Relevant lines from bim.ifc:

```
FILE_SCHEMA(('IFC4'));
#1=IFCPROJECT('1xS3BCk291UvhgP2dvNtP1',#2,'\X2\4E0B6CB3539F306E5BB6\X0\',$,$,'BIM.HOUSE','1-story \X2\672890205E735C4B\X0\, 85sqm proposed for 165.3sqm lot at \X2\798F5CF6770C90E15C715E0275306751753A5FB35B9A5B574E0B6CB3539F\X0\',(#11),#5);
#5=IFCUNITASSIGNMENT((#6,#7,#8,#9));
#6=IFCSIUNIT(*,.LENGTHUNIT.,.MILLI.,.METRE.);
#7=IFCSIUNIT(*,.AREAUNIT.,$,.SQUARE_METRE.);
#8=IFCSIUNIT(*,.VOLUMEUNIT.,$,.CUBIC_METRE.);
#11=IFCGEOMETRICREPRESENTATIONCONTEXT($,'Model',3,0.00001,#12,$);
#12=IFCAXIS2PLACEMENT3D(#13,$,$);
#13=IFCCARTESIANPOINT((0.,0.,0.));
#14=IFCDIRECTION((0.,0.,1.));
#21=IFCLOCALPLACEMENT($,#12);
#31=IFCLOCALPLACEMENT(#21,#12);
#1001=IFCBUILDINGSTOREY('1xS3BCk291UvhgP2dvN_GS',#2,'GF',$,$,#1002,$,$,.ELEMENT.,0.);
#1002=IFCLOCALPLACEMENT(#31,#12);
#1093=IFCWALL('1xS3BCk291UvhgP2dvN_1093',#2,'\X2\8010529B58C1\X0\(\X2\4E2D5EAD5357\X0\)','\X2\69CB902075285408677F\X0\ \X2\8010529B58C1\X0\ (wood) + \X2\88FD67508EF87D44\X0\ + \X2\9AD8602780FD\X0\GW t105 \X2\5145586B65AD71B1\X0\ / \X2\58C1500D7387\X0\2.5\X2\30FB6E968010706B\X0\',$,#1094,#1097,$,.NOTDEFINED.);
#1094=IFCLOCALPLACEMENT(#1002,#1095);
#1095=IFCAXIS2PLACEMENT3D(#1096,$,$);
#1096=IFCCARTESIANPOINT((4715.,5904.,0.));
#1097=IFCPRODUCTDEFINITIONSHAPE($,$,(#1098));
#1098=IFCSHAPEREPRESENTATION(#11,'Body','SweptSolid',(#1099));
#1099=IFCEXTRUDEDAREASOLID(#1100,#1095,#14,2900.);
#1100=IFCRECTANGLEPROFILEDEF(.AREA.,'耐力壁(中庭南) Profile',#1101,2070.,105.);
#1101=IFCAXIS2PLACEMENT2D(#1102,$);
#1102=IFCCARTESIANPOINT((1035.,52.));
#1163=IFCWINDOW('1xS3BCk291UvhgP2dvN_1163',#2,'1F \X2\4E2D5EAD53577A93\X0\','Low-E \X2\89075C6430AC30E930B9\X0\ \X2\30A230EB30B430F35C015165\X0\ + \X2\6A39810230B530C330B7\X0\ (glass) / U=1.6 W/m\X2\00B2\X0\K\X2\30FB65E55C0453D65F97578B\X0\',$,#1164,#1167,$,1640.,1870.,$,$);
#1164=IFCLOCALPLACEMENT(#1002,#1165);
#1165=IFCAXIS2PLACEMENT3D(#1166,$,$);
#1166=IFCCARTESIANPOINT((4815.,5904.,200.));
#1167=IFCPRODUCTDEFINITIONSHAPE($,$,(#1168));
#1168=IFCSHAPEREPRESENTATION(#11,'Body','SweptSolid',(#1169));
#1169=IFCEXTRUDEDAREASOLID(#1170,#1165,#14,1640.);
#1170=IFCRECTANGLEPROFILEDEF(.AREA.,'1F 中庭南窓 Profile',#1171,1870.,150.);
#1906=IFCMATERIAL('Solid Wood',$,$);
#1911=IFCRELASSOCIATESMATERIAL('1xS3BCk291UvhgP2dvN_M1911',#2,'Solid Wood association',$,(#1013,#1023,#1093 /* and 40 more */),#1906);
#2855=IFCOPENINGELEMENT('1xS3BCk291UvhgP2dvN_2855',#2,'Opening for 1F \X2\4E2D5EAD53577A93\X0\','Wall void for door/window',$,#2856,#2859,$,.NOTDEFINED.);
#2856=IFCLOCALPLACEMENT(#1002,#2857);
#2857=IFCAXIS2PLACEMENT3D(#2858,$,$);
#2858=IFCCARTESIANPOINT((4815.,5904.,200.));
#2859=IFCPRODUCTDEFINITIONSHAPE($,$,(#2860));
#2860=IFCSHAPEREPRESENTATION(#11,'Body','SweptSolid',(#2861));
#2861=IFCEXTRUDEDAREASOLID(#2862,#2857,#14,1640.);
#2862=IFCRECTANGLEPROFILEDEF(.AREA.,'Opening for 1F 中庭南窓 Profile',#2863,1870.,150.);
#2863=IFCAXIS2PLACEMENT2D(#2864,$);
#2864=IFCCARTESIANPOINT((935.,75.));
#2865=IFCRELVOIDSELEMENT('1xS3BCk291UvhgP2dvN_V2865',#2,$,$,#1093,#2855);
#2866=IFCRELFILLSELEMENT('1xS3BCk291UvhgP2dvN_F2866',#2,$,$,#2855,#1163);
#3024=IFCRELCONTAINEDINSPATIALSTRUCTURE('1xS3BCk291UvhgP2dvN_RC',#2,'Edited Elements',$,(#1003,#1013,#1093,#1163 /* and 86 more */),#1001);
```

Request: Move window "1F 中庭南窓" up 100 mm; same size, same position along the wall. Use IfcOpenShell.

```python
import numpy as np
import ifcopenshell
import ifcopenshell.api.geometry
import ifcopenshell.util.placement
import ifcopenshell.util.unit

model = ifcopenshell.open("bim.ifc")
unit_scale = ifcopenshell.util.unit.calculate_unit_scale(model)

window = model.by_id(1163)
opening = window.FillsVoids[0].RelatingOpeningElement
dz = 0.1 / unit_scale

shift = np.array([0.0, 0.0, dz])
# The window is not placed relative to its opening, so move both.
for product in (opening, window):
    matrix = ifcopenshell.util.placement.get_local_placement(product.ObjectPlacement)
    matrix[:3, 3] += shift
    ifcopenshell.api.geometry.edit_object_placement(model, product=product, matrix=matrix, is_si=False)

print(f"moved by {dz * unit_scale:+.3f} m")

model.write("bim_rev.ifc")
```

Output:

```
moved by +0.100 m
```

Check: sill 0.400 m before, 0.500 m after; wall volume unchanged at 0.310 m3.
